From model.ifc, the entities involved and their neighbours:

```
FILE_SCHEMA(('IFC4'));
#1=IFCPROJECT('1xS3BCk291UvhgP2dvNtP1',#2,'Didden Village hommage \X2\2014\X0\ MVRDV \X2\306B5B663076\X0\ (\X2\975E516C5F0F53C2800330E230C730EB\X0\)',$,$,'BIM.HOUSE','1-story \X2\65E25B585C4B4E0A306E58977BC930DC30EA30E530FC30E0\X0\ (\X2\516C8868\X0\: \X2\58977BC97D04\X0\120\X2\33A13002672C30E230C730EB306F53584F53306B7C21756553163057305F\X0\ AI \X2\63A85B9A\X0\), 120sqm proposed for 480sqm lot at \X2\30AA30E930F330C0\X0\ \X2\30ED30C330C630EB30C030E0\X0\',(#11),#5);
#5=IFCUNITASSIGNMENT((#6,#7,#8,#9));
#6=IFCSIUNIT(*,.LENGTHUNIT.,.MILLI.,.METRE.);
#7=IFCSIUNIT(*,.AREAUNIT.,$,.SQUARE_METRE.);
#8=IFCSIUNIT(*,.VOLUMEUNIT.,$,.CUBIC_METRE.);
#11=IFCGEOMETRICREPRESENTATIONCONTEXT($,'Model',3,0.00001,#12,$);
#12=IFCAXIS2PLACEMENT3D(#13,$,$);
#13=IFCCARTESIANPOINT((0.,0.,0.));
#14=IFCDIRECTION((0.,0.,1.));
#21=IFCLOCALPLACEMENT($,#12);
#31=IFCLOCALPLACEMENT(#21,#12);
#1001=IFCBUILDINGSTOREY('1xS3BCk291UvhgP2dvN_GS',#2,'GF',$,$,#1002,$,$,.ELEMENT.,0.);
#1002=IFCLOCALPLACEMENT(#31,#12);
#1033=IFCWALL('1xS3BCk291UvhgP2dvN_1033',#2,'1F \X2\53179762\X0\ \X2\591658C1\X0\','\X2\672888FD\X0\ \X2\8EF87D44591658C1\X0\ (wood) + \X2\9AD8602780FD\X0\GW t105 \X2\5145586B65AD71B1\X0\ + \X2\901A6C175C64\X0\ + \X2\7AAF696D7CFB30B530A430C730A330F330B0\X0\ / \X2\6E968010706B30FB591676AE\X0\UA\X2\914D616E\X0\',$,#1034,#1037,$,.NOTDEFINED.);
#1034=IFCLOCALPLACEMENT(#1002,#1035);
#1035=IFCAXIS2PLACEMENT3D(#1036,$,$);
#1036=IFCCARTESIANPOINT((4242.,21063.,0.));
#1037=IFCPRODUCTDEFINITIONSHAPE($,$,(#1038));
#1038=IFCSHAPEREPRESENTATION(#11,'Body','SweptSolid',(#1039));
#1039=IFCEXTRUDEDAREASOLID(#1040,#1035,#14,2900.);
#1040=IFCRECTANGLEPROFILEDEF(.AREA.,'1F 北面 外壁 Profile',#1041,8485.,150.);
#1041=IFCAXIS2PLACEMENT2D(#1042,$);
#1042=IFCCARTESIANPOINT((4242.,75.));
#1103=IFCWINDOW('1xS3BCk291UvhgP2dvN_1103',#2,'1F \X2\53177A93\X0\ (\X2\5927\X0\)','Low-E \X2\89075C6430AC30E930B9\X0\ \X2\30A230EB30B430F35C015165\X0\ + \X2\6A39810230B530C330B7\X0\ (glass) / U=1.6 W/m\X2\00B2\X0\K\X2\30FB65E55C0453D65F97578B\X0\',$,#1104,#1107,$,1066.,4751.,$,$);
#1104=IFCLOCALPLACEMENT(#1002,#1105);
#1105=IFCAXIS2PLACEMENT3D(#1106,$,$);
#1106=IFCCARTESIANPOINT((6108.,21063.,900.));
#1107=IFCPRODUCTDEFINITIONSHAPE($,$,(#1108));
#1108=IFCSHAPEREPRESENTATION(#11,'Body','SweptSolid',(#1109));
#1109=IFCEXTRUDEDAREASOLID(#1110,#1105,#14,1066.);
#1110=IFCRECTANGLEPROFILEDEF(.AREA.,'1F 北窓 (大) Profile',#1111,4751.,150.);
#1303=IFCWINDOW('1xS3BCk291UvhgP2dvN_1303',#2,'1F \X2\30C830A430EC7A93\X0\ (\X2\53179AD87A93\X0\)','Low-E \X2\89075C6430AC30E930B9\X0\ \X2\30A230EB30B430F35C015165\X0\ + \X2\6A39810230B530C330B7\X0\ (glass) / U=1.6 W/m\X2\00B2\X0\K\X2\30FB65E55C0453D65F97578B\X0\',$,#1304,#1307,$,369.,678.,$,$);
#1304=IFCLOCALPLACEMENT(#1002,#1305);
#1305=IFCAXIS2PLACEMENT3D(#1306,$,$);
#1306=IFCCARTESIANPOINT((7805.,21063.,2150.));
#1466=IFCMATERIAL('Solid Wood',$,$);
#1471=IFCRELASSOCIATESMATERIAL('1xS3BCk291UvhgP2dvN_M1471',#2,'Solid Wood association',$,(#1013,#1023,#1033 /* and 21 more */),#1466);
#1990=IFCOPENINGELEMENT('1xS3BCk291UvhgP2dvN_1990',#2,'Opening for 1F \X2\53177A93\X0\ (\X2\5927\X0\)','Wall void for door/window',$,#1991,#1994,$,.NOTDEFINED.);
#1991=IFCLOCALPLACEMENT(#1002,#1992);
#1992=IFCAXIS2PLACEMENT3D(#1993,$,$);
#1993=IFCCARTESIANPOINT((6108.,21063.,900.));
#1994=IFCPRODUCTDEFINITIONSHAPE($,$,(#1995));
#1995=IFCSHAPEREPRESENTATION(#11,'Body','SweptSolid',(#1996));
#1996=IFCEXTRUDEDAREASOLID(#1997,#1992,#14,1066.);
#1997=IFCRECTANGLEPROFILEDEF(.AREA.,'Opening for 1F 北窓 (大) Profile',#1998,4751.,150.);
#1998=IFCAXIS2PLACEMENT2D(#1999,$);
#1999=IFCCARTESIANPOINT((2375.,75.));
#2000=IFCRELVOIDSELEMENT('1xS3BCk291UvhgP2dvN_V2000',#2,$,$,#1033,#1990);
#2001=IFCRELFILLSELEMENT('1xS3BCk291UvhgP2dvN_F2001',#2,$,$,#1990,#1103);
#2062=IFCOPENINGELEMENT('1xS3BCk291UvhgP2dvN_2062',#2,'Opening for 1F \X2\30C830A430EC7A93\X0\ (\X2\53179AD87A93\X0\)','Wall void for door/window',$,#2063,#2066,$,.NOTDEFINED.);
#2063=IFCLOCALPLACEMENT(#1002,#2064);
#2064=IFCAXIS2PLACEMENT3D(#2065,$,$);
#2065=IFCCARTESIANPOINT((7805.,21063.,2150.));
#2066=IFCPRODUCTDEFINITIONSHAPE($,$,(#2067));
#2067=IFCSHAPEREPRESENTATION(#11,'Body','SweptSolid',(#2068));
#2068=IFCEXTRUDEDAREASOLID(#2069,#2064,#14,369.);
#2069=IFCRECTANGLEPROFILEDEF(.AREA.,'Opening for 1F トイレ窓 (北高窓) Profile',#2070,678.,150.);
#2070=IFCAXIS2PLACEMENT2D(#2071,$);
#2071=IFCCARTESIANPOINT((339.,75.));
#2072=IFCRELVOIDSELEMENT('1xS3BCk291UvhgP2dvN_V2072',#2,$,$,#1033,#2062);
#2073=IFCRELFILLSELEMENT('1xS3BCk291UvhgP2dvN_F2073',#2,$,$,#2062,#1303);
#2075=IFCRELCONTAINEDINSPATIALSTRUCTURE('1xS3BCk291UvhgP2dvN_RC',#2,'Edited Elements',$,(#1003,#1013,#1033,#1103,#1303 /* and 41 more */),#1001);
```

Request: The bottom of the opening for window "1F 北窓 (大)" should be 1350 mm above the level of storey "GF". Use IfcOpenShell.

```python
import numpy as np
import ifcopenshell
import ifcopenshell.api.geometry
import ifcopenshell.geom
import ifcopenshell.util.element
import ifcopenshell.util.placement
import ifcopenshell.util.shape
import ifcopenshell.util.unit

model = ifcopenshell.open("model.ifc")
unit_scale = ifcopenshell.util.unit.calculate_unit_scale(model)

window = model.by_guid("1xS3BCk291UvhgP2dvN_1103")
opening = window.FillsVoids[0].RelatingOpeningElement
storey = ifcopenshell.util.element.get_container(window, ifc_class="IfcBuildingStorey")
level = ifcopenshell.util.placement.get_local_placement(storey.ObjectPlacement)[2, 3]

# The opening's origin need not be at the sill, so measure its lowest point.
shape = ifcopenshell.geom.create_shape(ifcopenshell.geom.settings(), opening)
bottom = ifcopenshell.util.shape.get_shape_bottom_elevation(shape, shape.geometry) / unit_scale
dz = level + 1.35 / unit_scale - bottom

shift = np.array([0.0, 0.0, dz])
# The window is not placed relative to its opening, so move both.
for product in (opening, window):
    matrix = ifcopenshell.util.placement.get_local_placement(product.ObjectPlacement)
    matrix[:3, 3] += shift
    ifcopenshell.api.geometry.edit_object_placement(model, product=product, matrix=matrix, is_si=False)

print(f"moved by {dz * unit_scale:+.3f} m")

model.write("model_updated.ifc")
```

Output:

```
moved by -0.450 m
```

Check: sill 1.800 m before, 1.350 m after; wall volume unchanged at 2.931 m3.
